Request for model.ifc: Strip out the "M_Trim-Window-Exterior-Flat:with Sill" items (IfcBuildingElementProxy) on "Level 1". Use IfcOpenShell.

First a look at what the model holds.

```python
import ifcopenshell
import ifcopenshell.util.element

model = ifcopenshell.open("model.ifc")
print(model.schema)
storey = next(s for s in model.by_type("IfcBuildingStorey") if s.Name == "Level 1")
proxies = [e for e in ifcopenshell.util.element.get_decomposition(storey) if e.is_a("IfcBuildingElementProxy")]
seen = {}
for e in proxies:
    element_type = ifcopenshell.util.element.get_type(e)
    name = element_type.Name if element_type not in (None, e) else None
    seen[name] = seen.get(name, 0) + 1
for name, count in sorted(seen.items(), key=str):
    print(count, "x", name)
```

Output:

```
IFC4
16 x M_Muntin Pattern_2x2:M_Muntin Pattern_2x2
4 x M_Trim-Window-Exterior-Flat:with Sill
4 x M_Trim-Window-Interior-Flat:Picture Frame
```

```python
import ifcopenshell
import ifcopenshell.api.root
import ifcopenshell.util.element

model = ifcopenshell.open("model.ifc")

storey = next(s for s in model.by_type("IfcBuildingStorey") if s.Name == "Level 1")
proxies = [e for e in ifcopenshell.util.element.get_decomposition(storey) if e.is_a("IfcBuildingElementProxy")]
targets = [e for e in proxies if (t := ifcopenshell.util.element.get_type(e)) not in (None, e) and t.Name == "M_Trim-Window-Exterior-Flat:with Sill"]

for e in targets:
    ifcopenshell.api.root.remove_product(model, product=e)
print(len(targets), "removed")

model.write("model_edited.ifc")
```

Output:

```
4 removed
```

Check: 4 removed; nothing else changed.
